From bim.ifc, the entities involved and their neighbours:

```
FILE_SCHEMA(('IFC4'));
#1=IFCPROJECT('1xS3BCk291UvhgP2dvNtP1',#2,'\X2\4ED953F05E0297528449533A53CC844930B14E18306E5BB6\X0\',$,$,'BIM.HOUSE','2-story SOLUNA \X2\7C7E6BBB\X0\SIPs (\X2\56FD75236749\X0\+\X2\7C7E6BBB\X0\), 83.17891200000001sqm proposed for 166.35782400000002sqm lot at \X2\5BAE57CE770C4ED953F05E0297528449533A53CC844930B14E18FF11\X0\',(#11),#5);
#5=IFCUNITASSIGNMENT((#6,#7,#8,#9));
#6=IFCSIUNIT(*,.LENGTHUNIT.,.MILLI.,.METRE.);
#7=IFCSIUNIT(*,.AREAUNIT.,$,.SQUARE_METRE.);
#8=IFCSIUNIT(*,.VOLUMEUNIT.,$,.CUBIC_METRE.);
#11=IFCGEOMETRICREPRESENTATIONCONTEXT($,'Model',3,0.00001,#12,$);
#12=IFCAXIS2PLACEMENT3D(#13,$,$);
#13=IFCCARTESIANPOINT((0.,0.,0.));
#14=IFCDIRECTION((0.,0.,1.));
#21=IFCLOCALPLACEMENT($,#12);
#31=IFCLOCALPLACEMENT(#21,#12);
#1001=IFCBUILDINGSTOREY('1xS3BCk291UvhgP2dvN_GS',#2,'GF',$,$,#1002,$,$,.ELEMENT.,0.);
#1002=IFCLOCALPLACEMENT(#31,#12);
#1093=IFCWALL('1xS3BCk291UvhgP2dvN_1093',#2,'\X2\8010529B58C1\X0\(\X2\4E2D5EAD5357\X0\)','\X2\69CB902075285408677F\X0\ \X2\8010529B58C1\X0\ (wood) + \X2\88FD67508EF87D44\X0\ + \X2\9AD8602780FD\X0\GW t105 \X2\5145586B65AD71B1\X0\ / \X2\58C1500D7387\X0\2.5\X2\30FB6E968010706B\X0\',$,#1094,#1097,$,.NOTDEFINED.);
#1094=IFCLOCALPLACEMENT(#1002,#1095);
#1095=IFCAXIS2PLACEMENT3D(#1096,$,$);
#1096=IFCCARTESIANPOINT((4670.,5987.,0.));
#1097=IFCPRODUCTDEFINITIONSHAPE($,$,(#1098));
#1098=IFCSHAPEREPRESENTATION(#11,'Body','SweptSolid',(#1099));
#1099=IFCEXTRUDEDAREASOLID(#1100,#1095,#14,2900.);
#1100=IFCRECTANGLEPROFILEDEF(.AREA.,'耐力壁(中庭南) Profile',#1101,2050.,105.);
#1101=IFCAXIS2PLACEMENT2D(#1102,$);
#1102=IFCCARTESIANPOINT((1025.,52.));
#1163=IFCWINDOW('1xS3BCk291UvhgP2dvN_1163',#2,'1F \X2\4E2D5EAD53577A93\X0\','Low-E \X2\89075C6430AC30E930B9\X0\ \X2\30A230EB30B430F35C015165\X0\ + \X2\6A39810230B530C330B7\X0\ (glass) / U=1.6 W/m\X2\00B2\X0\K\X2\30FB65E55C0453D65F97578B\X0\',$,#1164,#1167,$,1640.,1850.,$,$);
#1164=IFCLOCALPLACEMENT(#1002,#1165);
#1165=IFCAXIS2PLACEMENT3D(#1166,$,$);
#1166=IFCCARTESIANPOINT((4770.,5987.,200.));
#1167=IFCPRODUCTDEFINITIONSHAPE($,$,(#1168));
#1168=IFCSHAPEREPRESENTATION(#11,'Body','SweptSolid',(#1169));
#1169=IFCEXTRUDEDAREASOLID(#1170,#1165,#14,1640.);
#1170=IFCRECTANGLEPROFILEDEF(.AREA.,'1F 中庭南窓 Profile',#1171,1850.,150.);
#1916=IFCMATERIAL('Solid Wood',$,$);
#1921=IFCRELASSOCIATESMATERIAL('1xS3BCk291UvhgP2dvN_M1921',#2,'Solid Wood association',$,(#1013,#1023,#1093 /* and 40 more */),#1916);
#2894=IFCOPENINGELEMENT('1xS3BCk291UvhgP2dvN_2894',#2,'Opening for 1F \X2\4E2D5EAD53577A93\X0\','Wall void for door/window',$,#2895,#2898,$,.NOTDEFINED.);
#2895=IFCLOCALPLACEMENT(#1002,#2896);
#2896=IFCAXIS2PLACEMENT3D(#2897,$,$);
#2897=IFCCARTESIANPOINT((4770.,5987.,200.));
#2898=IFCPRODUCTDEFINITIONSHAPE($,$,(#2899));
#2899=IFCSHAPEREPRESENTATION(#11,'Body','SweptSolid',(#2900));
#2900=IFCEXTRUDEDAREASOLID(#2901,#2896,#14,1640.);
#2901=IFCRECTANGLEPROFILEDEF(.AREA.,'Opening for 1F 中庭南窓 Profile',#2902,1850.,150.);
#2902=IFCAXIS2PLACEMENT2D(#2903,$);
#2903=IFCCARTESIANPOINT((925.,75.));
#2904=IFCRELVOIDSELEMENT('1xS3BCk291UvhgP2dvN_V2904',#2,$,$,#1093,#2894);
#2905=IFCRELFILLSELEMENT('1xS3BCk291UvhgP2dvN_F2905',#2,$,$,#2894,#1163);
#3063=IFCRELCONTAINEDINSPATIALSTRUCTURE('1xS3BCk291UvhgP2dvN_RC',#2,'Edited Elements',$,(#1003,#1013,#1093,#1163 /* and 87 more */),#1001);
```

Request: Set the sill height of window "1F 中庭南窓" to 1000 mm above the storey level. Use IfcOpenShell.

```python
import numpy as np
import ifcopenshell
import ifcopenshell.api.geometry
import ifcopenshell.geom
import ifcopenshell.util.element
import ifcopenshell.util.placement
import ifcopenshell.util.shape
import ifcopenshell.util.unit

model = ifcopenshell.open("bim.ifc")
unit_scale = ifcopenshell.util.unit.calculate_unit_scale(model)

window = model.by_guid("1xS3BCk291UvhgP2dvN_1163")
opening = window.FillsVoids[0].RelatingOpeningElement
storey = ifcopenshell.util.element.get_container(window, ifc_class="IfcBuildingStorey")
level = ifcopenshell.util.placement.get_local_placement(storey.ObjectPlacement)[2, 3]

# The opening's origin need not be at the sill, so measure its lowest point.
shape = ifcopenshell.geom.create_shape(ifcopenshell.geom.settings(), opening)
bottom = ifcopenshell.util.shape.get_shape_bottom_elevation(shape, shape.geometry) / unit_scale
dz = level + 1000.0 - bottom

shift = np.array([0.0, 0.0, dz])
# The window is not placed relative to its opening, so move both.
for product in (opening, window):
    matrix = ifcopenshell.util.placement.get_local_placement(product.ObjectPlacement)
    matrix[:3, 3] += shift
    ifcopenshell.api.geometry.edit_object_placement(model, product=product, matrix=matrix, is_si=False)

print(f"moved by {dz * unit_scale:+.3f} m")

model.write("bim_edited.ifc")
```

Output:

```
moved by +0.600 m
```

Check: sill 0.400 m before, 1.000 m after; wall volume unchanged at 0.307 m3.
